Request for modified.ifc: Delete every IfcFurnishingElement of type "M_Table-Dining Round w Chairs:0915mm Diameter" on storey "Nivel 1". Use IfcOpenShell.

First a look at what the model holds.

```python
import ifcopenshell
import ifcopenshell.util.element

model = ifcopenshell.open("modified.ifc")
print(model.schema)
storey = next(s for s in model.by_type("IfcBuildingStorey") if s.Name == "Nivel 1")
furniture = [e for e in ifcopenshell.util.element.get_decomposition(storey) if e.is_a("IfcFurnishingElement")]
seen = {}
for e in furniture:
    element_type = ifcopenshell.util.element.get_type(e)
    name = element_type.Name if element_type not in (None, e) else None
    seen[name] = seen.get(name, 0) + 1
for name, count in sorted(seen.items(), key=str):
    print(count, "x", name)
```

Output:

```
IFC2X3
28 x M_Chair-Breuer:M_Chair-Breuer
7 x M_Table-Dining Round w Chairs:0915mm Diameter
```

```python
import ifcopenshell
import ifcopenshell.api.root
import ifcopenshell.util.element

model = ifcopenshell.open("modified.ifc")

storey = next(s for s in model.by_type("IfcBuildingStorey") if s.Name == "Nivel 1")
furniture = [e for e in ifcopenshell.util.element.get_decomposition(storey) if e.is_a("IfcFurnishingElement")]
targets = [e for e in furniture if (t := ifcopenshell.util.element.get_type(e)) not in (None, e) and t.Name == "M_Table-Dining Round w Chairs:0915mm Diameter"]

for e in targets:
    ifcopenshell.api.root.remove_product(model, product=e)
print(len(targets), "removed")

model.write("modified_rev.ifc")
```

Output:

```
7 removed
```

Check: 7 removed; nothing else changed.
